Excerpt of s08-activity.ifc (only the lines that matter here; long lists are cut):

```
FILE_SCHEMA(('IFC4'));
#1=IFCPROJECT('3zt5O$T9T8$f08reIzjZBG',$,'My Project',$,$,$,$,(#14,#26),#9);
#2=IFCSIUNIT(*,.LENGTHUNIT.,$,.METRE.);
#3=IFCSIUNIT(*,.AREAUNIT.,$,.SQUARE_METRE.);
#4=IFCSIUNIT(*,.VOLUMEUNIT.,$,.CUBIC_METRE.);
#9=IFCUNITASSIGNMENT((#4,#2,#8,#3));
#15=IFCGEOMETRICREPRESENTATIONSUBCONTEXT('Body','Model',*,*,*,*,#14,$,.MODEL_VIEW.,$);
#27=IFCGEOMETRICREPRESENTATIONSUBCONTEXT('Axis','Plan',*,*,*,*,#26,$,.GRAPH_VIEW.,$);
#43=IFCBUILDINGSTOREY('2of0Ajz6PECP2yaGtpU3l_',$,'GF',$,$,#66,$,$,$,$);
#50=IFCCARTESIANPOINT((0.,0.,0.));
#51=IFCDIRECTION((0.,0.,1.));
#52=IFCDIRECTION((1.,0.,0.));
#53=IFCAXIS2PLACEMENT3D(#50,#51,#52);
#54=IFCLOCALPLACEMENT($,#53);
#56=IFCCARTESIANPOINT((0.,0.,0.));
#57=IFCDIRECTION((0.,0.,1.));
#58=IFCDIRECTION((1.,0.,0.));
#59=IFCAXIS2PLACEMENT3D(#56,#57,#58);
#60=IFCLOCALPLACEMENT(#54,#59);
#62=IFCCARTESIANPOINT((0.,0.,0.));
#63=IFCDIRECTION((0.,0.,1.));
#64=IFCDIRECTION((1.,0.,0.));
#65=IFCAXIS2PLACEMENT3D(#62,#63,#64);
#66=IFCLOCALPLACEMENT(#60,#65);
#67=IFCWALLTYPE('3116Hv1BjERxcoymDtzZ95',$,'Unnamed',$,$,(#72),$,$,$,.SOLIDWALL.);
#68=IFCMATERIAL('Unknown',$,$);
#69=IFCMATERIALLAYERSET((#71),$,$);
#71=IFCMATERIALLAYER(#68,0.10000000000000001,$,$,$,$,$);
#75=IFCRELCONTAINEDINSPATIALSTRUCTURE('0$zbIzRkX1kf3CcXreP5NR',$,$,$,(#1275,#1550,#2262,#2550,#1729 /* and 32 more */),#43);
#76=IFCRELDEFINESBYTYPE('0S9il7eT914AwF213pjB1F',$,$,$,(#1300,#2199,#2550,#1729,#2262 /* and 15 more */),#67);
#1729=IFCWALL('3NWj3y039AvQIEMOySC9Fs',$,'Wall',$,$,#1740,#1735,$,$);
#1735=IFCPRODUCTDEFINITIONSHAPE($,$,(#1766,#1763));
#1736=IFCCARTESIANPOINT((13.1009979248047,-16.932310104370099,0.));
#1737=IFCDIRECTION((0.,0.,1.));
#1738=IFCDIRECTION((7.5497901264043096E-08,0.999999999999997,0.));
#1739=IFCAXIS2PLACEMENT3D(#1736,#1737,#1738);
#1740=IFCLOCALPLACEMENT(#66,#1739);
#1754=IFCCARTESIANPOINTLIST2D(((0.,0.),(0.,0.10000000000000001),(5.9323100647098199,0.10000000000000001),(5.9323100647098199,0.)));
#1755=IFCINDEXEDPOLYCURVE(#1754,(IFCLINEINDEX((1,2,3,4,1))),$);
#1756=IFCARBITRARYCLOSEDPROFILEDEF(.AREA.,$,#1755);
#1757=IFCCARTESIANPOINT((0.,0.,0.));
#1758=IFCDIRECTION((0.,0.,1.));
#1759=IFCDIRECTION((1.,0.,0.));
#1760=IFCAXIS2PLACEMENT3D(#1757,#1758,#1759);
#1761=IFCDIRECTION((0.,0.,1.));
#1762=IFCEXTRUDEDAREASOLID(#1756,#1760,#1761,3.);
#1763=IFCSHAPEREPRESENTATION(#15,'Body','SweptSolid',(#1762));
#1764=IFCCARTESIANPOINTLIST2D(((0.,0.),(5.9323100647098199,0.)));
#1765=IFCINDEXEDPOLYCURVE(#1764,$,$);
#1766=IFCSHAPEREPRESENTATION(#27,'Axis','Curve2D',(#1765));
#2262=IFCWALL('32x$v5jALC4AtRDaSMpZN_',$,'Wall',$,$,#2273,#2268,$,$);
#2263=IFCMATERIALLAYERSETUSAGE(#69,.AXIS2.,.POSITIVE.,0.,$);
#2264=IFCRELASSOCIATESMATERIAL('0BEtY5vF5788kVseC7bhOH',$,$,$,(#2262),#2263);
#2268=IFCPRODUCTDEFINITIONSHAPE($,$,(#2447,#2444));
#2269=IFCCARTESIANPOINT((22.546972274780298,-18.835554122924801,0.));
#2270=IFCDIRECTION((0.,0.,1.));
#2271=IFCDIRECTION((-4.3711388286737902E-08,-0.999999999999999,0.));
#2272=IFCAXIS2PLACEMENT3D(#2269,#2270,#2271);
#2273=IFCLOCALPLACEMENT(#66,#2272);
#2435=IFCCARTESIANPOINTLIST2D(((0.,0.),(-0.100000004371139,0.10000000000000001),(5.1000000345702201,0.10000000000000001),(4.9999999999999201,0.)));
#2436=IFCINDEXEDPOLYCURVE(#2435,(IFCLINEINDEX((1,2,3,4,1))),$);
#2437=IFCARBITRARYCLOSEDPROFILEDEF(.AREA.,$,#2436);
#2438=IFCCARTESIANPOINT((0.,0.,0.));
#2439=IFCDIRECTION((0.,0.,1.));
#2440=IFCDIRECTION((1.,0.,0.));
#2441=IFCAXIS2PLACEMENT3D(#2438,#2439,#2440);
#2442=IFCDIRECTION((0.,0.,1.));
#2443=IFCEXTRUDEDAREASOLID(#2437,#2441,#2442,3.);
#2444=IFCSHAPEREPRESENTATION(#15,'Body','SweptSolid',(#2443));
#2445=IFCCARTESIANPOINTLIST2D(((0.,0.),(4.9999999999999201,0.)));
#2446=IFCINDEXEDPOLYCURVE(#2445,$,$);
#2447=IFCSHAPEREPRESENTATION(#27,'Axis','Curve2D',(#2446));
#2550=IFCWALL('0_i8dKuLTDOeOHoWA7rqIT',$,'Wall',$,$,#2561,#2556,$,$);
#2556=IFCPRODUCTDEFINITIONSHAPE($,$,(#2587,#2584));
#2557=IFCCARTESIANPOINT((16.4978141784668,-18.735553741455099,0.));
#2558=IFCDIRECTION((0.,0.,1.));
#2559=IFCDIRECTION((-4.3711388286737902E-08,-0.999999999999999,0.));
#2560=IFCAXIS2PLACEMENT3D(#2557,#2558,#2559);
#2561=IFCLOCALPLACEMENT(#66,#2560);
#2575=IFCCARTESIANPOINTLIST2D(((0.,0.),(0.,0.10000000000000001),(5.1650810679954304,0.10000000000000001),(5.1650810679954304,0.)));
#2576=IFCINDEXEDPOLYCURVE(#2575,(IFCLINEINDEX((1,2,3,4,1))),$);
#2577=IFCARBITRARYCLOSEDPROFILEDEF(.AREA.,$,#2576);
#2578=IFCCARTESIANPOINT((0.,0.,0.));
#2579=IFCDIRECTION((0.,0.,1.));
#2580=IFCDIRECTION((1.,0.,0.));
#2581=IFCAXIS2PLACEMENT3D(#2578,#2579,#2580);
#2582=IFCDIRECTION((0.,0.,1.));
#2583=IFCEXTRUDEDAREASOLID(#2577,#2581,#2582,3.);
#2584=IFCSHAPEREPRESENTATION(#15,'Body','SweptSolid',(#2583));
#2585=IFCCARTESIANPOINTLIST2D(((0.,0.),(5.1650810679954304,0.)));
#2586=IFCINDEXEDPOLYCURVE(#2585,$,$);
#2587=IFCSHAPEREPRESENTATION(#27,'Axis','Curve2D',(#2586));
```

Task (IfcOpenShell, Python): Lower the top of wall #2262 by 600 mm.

```python
import ifcopenshell
import ifcopenshell.geom
import ifcopenshell.util.representation
import ifcopenshell.util.shape

model = ifcopenshell.open("s08-activity.ifc")
settings = ifcopenshell.geom.settings()


def volume(element):
    """Net volume in cubic metres, openings subtracted."""
    shape = ifcopenshell.geom.create_shape(settings, element)
    return ifcopenshell.util.shape.get_volume(shape.geometry)


wall = model.by_guid("32x$v5jALC4AtRDaSMpZN_")
before = volume(wall)

body = ifcopenshell.util.representation.get_representation(wall, "Model", "Body")
solid = body.Items[0]
old_height = solid.Depth
solid.Depth -= 0.6
after = volume(wall)

print(f"height {old_height:g} -> {solid.Depth:g}, volume {before:.3f} -> {after:.3f} m3")

model.write("s08-activity_edited.ifc")
```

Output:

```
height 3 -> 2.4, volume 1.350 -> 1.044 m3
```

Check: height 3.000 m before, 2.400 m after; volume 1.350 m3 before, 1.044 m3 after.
